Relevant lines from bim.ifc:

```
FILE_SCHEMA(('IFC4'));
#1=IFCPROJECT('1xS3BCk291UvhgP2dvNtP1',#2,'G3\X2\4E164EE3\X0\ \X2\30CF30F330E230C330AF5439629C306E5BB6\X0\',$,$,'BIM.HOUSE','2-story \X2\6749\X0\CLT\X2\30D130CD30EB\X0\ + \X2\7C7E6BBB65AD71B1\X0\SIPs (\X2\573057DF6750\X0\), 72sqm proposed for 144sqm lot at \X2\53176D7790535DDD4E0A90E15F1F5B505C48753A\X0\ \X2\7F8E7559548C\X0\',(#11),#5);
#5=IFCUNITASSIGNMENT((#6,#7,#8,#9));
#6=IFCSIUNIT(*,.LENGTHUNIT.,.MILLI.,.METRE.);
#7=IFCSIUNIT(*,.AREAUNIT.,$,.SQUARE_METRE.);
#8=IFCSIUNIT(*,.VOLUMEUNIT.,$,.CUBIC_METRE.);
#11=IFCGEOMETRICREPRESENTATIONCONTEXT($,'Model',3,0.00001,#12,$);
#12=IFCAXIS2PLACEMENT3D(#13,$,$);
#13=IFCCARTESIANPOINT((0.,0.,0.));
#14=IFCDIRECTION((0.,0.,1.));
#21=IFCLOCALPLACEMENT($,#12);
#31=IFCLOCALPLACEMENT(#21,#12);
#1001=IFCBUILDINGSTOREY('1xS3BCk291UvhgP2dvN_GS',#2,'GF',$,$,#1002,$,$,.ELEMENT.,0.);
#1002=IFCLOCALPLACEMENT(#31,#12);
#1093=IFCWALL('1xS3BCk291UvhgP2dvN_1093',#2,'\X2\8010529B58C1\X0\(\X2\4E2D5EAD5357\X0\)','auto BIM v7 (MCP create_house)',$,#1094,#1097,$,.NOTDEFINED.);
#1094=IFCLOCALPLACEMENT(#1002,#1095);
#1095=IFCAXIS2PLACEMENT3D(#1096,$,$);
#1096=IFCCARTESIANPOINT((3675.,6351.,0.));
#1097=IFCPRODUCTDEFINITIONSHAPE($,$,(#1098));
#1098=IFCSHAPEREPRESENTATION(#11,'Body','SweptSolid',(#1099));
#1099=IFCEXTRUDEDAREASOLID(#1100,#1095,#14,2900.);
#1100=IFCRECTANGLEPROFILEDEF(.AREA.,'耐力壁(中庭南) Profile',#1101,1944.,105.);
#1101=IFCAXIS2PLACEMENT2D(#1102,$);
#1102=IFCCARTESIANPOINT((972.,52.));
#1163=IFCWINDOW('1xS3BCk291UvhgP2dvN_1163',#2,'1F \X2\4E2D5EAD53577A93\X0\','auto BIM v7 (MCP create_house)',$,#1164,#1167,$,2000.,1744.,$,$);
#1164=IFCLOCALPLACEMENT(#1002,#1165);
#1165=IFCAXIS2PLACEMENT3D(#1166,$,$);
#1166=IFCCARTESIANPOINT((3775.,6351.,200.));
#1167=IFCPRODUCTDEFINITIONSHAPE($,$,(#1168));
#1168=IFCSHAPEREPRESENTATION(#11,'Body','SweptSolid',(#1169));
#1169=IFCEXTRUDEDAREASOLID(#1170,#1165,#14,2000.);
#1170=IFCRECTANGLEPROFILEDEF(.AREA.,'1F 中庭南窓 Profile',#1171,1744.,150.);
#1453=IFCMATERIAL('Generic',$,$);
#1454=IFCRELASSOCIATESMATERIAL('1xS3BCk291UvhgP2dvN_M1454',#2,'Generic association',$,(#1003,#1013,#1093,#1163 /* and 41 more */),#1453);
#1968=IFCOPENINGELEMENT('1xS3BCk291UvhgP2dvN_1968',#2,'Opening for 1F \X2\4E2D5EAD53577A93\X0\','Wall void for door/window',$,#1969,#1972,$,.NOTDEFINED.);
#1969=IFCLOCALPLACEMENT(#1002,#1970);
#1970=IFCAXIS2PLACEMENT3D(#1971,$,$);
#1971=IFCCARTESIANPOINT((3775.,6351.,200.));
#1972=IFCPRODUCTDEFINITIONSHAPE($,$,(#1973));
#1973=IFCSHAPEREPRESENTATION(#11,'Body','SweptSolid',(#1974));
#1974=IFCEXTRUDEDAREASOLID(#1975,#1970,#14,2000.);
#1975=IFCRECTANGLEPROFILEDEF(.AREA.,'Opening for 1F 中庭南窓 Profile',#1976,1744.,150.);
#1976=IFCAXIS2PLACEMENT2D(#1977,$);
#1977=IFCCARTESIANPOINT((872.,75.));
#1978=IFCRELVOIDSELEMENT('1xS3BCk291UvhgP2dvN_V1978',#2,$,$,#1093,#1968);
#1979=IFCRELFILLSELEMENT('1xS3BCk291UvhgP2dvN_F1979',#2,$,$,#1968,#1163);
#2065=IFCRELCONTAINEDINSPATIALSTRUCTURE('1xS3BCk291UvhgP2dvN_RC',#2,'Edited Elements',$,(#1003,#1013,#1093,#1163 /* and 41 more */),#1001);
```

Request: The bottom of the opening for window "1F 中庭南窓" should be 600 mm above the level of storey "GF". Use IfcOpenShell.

```python
import numpy as np
import ifcopenshell
import ifcopenshell.api.geometry
import ifcopenshell.geom
import ifcopenshell.util.element
import ifcopenshell.util.placement
import ifcopenshell.util.shape
import ifcopenshell.util.unit

model = ifcopenshell.open("bim.ifc")
unit_scale = ifcopenshell.util.unit.calculate_unit_scale(model)

window = model.by_guid("1xS3BCk291UvhgP2dvN_1163")
opening = window.FillsVoids[0].RelatingOpeningElement
storey = ifcopenshell.util.element.get_container(window, ifc_class="IfcBuildingStorey")
level = ifcopenshell.util.placement.get_local_placement(storey.ObjectPlacement)[2, 3]

# The opening's origin need not be at the sill, so measure its lowest point.
shape = ifcopenshell.geom.create_shape(ifcopenshell.geom.settings(), opening)
bottom = ifcopenshell.util.shape.get_shape_bottom_elevation(shape, shape.geometry) / unit_scale
dz = level + 600.0 - bottom

shift = np.array([0.0, 0.0, dz])
# The window is not placed relative to its opening, so move both.
for product in (opening, window):
    matrix = ifcopenshell.util.placement.get_local_placement(product.ObjectPlacement)
    matrix[:3, 3] += shift
    ifcopenshell.api.geometry.edit_object_placement(model, product=product, matrix=matrix, is_si=False)

print(f"moved by {dz * unit_scale:+.3f} m")

model.write("bim_updated.ifc")
```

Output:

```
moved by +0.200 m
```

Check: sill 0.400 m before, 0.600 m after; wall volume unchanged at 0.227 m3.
